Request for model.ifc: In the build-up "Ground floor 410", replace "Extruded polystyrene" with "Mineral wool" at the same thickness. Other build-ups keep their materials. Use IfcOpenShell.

First a look at what the model holds.

```python
import ifcopenshell
import ifcopenshell.util.element

model = ifcopenshell.open("model.ifc")
print(model.schema)
for layer_set in model.by_type("IfcMaterialLayerSet"):
    if layer_set.LayerSetName == "Ground floor 410":
        for layer in layer_set.MaterialLayers:
            print(layer.id(), layer.Material and layer.Material.Name, layer.LayerThickness, sep=" | ")
        print(len(ifcopenshell.util.element.get_elements_by_material(model, layer_set)), "elements and types use it")
print(sorted(m.Name for m in model.by_type("IfcMaterial") if m.Name)[:60])
```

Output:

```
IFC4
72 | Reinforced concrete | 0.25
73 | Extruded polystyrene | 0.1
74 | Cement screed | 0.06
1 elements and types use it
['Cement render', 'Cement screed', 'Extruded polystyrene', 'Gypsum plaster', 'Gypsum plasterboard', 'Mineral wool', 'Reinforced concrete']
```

```python
import ifcopenshell
import ifcopenshell.api.material

model = ifcopenshell.open("model.ifc")

layer_set = next(s for s in model.by_type("IfcMaterialLayerSet") if s.LayerSetName == "Ground floor 410")
layer = next(l for l in layer_set.MaterialLayers if l.Material and l.Material.Name == "Extruded polystyrene")
material = next(m for m in model.by_type("IfcMaterial") if m.Name == "Mineral wool")

# Point this one layer at the other material; renaming the old one would change it everywhere.
ifcopenshell.api.material.edit_layer(model, layer=layer, attributes={"Name": material.Name}, material=material)

print([l.Material.Name if l.Material else None for l in layer_set.MaterialLayers])

model.write("model_v2.ifc")
```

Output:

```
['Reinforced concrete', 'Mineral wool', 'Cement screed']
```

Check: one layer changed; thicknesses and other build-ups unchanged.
